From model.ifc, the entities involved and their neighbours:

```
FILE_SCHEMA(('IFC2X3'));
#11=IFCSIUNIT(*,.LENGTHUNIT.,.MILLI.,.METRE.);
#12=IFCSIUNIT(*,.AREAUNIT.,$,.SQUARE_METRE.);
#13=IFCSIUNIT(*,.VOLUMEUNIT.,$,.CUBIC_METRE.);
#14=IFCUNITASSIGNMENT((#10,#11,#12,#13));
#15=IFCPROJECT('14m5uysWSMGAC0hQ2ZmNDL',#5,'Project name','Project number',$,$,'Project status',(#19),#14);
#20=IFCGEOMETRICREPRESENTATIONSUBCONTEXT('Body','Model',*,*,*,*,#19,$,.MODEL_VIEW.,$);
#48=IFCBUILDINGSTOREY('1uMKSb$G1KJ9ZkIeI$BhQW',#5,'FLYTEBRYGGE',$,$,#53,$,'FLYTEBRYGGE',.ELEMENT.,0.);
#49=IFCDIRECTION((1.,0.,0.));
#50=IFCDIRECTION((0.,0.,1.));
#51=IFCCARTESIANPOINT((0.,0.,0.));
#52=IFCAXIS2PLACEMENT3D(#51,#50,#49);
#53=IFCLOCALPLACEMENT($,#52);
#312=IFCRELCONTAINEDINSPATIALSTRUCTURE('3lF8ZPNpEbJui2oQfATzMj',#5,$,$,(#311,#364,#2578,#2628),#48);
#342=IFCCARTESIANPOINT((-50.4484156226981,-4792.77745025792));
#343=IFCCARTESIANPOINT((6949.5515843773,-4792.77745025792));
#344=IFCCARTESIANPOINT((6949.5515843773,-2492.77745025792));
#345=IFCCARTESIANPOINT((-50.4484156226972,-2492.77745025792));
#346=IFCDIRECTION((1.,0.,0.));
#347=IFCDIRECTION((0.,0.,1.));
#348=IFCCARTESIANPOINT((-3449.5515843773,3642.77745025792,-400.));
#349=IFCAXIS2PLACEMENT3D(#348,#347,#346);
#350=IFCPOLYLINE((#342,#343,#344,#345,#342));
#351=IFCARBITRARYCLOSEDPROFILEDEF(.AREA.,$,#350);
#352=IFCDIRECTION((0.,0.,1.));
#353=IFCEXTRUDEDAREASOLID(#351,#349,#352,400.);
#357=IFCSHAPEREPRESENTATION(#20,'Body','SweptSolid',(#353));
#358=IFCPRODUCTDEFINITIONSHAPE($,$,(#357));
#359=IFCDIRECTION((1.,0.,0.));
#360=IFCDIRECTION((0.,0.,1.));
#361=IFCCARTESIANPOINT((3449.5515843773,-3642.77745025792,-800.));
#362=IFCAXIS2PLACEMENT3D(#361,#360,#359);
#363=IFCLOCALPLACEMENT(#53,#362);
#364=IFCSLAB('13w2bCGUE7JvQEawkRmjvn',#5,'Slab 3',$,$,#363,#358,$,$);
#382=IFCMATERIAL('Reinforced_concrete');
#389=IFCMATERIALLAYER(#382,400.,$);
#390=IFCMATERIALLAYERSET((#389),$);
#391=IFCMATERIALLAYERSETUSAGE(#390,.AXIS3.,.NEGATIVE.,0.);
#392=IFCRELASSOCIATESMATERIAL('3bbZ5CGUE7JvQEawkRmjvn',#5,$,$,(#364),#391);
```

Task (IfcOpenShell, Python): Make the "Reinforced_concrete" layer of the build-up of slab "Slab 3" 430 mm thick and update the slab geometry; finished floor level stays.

```python
import ifcopenshell
import ifcopenshell.util.element
import ifcopenshell.util.representation

model = ifcopenshell.open("model.ifc")

layer_set = model.by_id(390)
layer = next(l for l in layer_set.MaterialLayers if l.Material and l.Material.Name == "Reinforced_concrete")
change = 430.0 - layer.LayerThickness
layer.LayerThickness += change

# Geometry does not follow the layer set by itself.
slabs = [e for e in ifcopenshell.util.element.get_elements_by_material(model, layer_set) if e.is_a("IfcSlab")]
for slab in sorted(slabs, key=lambda e: e.id()):
    body = ifcopenshell.util.representation.get_representation(slab, "Model", "Body")
    solid = body.Items[0]
    old_depth = solid.Depth
    solid.Depth += change
    # Extruded upwards: lower the start of the extrusion so the top stays.
    x, y, z = solid.Position.Location.Coordinates
    solid.Position.Location = model.createIfcCartesianPoint((x, y, z - change))
    print(slab.id(), f"{old_depth:g} -> {solid.Depth:g}")

model.write("model_updated.ifc")
```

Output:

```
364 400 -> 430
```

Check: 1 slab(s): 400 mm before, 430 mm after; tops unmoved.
